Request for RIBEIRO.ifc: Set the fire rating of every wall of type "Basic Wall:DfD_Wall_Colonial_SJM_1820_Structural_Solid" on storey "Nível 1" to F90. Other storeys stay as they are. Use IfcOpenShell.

First a look at what the model holds.

```python
import ifcopenshell
import ifcopenshell.util.element

model = ifcopenshell.open("RIBEIRO.ifc")
print(model.schema)
storey = next(s for s in model.by_type("IfcBuildingStorey") if s.Name == "Nível 1")
walls = [e for e in ifcopenshell.util.element.get_decomposition(storey) if e.is_a("IfcWall")]
seen = {}
for e in walls:
    element_type = ifcopenshell.util.element.get_type(e)
    key = (element_type.Name if element_type != e and element_type else None, ifcopenshell.util.element.get_pset(e, "Pset_WallCommon", "FireRating"))
    seen[key] = seen.get(key, 0) + 1
for (name, value), count in sorted(seen.items(), key=str):
    print(count, "x", name, "|", value)
```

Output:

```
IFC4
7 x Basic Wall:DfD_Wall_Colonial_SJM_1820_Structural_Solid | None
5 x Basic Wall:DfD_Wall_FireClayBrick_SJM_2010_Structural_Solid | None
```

```python
import ifcopenshell
import ifcopenshell.api.pset
import ifcopenshell.util.element

model = ifcopenshell.open("RIBEIRO.ifc")

storey = next(s for s in model.by_type("IfcBuildingStorey") if s.Name == "Nível 1")
walls = [e for e in ifcopenshell.util.element.get_decomposition(storey) if e.is_a("IfcWall")]

count = 0
for e in walls:
    element_type = ifcopenshell.util.element.get_type(e)
    if element_type in (None, e) or element_type.Name != "Basic Wall:DfD_Wall_Colonial_SJM_1820_Structural_Solid":
        continue
    # add_pset returns the element's existing set when there is one.
    pset = ifcopenshell.api.pset.add_pset(model, product=e, name="Pset_WallCommon")
    ifcopenshell.api.pset.edit_pset(model, pset=pset, properties={"FireRating": "F90"})
    count += 1

print(count, "walls updated")

model.write("RIBEIRO-out.ifc")
```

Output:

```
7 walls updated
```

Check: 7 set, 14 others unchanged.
